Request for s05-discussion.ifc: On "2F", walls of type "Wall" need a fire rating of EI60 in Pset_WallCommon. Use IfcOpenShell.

First a look at what the model holds.

```python
import ifcopenshell
import ifcopenshell.util.element

model = ifcopenshell.open("s05-discussion.ifc")
print(model.schema)
storey = next(s for s in model.by_type("IfcBuildingStorey") if s.Name == "2F")
walls = [e for e in ifcopenshell.util.element.get_decomposition(storey) if e.is_a("IfcWall")]
seen = {}
for e in walls:
    element_type = ifcopenshell.util.element.get_type(e)
    key = (element_type.Name if element_type != e and element_type else None, ifcopenshell.util.element.get_pset(e, "Pset_WallCommon", "FireRating"))
    seen[key] = seen.get(key, 0) + 1
for (name, value), count in sorted(seen.items(), key=str):
    print(count, "x", name, "|", value)
```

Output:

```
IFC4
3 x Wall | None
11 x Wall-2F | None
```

```python
import ifcopenshell
import ifcopenshell.api.pset
import ifcopenshell.util.element

model = ifcopenshell.open("s05-discussion.ifc")

storey = next(s for s in model.by_type("IfcBuildingStorey") if s.Name == "2F")
walls = [e for e in ifcopenshell.util.element.get_decomposition(storey) if e.is_a("IfcWall")]

count = 0
for e in walls:
    element_type = ifcopenshell.util.element.get_type(e)
    if element_type in (None, e) or element_type.Name != "Wall":
        continue
    # add_pset returns the element's existing set when there is one.
    pset = ifcopenshell.api.pset.add_pset(model, product=e, name="Pset_WallCommon")
    ifcopenshell.api.pset.edit_pset(model, pset=pset, properties={"FireRating": "EI60"})
    count += 1

print(count, "walls updated")

model.write("s05-discussion_updated.ifc")
```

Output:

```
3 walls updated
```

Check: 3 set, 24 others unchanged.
